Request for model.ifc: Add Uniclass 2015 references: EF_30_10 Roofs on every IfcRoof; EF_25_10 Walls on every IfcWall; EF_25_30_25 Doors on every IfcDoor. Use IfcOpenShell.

First a look at what the model holds.

```python
import ifcopenshell

model = ifcopenshell.open("model.ifc")
print(model.schema)
print("classifications:", [c.Name for c in model.by_type("IfcClassification")])
for ifc_class in ("IfcDoor", "IfcRoof", "IfcStair", "IfcWall", "IfcWindow"):
    print(ifc_class, len(model.by_type(ifc_class)))
```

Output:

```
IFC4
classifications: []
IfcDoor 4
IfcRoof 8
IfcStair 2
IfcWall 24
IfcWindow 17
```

```python
import ifcopenshell
import ifcopenshell.api.classification

model = ifcopenshell.open("model.ifc")

system = ifcopenshell.api.classification.add_classification(model, classification="Uniclass 2015")

codes = {
    "IfcRoof": ("EF_30_10", "Roofs"),
    "IfcWall": ("EF_25_10", "Walls"),
    "IfcDoor": ("EF_25_30_25", "Doors"),
}
for ifc_class, (code, name) in codes.items():
    products = model.by_type(ifc_class)
    ifcopenshell.api.classification.add_reference(
        model, products=products, classification=system, identification=code, name=name
    )
    print(code, len(products))

model.write("model_edited.ifc")
```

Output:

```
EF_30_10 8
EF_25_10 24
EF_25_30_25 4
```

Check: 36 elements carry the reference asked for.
